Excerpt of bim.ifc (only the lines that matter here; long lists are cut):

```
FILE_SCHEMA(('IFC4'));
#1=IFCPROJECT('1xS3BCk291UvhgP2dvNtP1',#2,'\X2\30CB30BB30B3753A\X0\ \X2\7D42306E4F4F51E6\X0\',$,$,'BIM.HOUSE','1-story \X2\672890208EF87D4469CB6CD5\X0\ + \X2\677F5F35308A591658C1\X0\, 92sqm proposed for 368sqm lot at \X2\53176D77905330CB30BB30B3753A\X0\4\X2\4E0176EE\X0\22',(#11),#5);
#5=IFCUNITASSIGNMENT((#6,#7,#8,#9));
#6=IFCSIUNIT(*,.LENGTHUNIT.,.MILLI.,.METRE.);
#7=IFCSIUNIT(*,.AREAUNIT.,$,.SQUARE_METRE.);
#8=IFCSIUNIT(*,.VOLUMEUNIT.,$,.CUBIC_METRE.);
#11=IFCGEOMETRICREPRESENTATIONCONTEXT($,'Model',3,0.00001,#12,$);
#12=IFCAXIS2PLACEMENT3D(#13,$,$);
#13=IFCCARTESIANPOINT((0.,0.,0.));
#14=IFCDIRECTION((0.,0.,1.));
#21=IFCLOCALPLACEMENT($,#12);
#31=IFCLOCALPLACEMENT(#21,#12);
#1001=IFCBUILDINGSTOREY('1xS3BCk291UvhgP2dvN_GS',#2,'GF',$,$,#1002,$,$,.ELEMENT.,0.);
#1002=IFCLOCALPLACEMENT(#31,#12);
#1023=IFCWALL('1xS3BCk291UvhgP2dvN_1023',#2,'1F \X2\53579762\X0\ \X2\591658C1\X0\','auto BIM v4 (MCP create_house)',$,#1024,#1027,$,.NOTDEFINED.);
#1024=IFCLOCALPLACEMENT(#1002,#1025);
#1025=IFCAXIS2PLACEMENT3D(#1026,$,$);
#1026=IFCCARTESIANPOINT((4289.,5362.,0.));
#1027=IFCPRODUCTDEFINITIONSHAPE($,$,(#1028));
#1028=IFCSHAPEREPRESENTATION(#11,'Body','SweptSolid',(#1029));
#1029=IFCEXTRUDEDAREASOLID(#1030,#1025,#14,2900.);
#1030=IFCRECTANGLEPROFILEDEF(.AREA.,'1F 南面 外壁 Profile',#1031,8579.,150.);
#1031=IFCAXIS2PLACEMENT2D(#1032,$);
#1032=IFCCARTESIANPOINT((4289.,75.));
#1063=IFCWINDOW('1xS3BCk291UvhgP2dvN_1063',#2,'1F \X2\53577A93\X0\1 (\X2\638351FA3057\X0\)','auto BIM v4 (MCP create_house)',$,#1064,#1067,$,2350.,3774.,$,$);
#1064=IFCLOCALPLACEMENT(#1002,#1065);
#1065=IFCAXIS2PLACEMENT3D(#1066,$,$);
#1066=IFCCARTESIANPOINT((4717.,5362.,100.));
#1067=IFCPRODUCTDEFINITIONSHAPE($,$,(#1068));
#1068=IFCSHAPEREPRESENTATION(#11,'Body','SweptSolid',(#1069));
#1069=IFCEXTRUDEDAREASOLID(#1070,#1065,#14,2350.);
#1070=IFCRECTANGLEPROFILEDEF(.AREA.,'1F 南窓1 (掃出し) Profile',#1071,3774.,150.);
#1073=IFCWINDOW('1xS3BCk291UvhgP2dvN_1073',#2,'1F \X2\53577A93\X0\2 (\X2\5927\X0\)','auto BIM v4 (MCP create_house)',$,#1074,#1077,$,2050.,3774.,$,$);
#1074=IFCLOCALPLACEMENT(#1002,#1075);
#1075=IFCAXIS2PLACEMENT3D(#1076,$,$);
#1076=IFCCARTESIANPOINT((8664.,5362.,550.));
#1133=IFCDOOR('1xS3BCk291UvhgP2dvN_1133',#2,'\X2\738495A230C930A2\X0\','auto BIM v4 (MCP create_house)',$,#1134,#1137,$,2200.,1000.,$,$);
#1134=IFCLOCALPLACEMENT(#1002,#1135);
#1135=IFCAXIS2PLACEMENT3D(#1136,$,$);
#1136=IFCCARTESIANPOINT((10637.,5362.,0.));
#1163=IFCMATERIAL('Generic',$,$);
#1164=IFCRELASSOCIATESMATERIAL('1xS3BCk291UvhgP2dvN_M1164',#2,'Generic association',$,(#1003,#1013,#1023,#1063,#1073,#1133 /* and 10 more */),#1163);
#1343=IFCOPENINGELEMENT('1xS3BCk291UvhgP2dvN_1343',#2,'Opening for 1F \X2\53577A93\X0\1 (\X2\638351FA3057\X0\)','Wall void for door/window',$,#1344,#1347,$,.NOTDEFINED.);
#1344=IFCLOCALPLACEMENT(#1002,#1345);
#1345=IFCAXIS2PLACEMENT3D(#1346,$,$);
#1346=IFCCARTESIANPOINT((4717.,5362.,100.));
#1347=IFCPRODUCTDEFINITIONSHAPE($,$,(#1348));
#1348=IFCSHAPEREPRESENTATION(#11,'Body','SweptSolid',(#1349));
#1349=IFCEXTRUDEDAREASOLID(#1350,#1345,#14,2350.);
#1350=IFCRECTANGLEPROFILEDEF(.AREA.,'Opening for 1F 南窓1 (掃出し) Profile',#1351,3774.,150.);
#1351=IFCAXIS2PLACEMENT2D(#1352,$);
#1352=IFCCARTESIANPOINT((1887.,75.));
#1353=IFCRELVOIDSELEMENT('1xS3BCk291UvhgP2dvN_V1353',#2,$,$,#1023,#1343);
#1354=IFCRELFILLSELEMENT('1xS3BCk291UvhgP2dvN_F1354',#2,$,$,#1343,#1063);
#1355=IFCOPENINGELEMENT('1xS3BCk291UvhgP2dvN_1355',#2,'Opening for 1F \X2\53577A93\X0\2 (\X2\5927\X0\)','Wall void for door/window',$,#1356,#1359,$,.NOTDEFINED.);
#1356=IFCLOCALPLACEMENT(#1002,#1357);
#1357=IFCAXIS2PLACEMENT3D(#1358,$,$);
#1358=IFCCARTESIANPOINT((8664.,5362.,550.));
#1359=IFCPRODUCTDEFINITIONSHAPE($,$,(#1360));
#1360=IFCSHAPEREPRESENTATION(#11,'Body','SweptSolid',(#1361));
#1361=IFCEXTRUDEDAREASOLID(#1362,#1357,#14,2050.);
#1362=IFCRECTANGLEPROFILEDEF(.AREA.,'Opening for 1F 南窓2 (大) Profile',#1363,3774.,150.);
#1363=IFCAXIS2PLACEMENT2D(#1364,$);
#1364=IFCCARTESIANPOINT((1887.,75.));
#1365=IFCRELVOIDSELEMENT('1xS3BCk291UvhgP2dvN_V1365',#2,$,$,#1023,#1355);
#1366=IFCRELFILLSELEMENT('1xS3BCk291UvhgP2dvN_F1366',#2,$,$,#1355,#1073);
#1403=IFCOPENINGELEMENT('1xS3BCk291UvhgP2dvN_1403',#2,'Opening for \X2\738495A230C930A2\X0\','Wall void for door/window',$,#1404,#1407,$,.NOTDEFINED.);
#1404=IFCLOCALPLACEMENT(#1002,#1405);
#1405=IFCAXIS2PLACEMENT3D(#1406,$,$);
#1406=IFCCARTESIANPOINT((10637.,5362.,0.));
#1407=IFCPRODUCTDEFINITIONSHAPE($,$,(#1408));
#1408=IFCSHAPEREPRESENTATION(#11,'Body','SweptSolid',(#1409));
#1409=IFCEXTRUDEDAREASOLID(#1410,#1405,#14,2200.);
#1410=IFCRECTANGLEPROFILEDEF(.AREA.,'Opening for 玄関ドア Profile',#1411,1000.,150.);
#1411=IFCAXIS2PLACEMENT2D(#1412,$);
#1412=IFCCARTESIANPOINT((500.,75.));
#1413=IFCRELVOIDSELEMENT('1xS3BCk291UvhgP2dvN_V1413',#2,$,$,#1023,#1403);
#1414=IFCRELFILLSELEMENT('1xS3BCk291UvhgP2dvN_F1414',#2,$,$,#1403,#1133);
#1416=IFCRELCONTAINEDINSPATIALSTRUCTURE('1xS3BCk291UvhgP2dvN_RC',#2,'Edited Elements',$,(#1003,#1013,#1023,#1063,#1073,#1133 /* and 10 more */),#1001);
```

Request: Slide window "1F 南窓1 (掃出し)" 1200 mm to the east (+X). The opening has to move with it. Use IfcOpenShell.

```python
import ifcopenshell
import ifcopenshell.api.geometry
import ifcopenshell.util.placement

model = ifcopenshell.open("bim.ifc")

window = model.by_guid("1xS3BCk291UvhgP2dvN_1063")
opening = window.FillsVoids[0].RelatingOpeningElement
wall = opening.VoidsElements[0].RelatingBuildingElement

wall_matrix = ifcopenshell.util.placement.get_local_placement(wall.ObjectPlacement)
shift = wall_matrix[:3, 0] * 1200.0
before = ifcopenshell.util.placement.get_local_placement(window.ObjectPlacement)[:3, 3].copy()

# The window is not placed relative to its opening, so move both.
for product in (opening, window):
    matrix = ifcopenshell.util.placement.get_local_placement(product.ObjectPlacement)
    matrix[:3, 3] += shift
    ifcopenshell.api.geometry.edit_object_placement(model, product=product, matrix=matrix, is_si=False)

after = ifcopenshell.util.placement.get_local_placement(window.ObjectPlacement)[:3, 3]
print("window moved by", (after - before).round(3) + 0.0)

model.write("bim_updated.ifc")
```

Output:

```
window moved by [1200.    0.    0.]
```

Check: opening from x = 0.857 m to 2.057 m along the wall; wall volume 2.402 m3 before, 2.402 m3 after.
